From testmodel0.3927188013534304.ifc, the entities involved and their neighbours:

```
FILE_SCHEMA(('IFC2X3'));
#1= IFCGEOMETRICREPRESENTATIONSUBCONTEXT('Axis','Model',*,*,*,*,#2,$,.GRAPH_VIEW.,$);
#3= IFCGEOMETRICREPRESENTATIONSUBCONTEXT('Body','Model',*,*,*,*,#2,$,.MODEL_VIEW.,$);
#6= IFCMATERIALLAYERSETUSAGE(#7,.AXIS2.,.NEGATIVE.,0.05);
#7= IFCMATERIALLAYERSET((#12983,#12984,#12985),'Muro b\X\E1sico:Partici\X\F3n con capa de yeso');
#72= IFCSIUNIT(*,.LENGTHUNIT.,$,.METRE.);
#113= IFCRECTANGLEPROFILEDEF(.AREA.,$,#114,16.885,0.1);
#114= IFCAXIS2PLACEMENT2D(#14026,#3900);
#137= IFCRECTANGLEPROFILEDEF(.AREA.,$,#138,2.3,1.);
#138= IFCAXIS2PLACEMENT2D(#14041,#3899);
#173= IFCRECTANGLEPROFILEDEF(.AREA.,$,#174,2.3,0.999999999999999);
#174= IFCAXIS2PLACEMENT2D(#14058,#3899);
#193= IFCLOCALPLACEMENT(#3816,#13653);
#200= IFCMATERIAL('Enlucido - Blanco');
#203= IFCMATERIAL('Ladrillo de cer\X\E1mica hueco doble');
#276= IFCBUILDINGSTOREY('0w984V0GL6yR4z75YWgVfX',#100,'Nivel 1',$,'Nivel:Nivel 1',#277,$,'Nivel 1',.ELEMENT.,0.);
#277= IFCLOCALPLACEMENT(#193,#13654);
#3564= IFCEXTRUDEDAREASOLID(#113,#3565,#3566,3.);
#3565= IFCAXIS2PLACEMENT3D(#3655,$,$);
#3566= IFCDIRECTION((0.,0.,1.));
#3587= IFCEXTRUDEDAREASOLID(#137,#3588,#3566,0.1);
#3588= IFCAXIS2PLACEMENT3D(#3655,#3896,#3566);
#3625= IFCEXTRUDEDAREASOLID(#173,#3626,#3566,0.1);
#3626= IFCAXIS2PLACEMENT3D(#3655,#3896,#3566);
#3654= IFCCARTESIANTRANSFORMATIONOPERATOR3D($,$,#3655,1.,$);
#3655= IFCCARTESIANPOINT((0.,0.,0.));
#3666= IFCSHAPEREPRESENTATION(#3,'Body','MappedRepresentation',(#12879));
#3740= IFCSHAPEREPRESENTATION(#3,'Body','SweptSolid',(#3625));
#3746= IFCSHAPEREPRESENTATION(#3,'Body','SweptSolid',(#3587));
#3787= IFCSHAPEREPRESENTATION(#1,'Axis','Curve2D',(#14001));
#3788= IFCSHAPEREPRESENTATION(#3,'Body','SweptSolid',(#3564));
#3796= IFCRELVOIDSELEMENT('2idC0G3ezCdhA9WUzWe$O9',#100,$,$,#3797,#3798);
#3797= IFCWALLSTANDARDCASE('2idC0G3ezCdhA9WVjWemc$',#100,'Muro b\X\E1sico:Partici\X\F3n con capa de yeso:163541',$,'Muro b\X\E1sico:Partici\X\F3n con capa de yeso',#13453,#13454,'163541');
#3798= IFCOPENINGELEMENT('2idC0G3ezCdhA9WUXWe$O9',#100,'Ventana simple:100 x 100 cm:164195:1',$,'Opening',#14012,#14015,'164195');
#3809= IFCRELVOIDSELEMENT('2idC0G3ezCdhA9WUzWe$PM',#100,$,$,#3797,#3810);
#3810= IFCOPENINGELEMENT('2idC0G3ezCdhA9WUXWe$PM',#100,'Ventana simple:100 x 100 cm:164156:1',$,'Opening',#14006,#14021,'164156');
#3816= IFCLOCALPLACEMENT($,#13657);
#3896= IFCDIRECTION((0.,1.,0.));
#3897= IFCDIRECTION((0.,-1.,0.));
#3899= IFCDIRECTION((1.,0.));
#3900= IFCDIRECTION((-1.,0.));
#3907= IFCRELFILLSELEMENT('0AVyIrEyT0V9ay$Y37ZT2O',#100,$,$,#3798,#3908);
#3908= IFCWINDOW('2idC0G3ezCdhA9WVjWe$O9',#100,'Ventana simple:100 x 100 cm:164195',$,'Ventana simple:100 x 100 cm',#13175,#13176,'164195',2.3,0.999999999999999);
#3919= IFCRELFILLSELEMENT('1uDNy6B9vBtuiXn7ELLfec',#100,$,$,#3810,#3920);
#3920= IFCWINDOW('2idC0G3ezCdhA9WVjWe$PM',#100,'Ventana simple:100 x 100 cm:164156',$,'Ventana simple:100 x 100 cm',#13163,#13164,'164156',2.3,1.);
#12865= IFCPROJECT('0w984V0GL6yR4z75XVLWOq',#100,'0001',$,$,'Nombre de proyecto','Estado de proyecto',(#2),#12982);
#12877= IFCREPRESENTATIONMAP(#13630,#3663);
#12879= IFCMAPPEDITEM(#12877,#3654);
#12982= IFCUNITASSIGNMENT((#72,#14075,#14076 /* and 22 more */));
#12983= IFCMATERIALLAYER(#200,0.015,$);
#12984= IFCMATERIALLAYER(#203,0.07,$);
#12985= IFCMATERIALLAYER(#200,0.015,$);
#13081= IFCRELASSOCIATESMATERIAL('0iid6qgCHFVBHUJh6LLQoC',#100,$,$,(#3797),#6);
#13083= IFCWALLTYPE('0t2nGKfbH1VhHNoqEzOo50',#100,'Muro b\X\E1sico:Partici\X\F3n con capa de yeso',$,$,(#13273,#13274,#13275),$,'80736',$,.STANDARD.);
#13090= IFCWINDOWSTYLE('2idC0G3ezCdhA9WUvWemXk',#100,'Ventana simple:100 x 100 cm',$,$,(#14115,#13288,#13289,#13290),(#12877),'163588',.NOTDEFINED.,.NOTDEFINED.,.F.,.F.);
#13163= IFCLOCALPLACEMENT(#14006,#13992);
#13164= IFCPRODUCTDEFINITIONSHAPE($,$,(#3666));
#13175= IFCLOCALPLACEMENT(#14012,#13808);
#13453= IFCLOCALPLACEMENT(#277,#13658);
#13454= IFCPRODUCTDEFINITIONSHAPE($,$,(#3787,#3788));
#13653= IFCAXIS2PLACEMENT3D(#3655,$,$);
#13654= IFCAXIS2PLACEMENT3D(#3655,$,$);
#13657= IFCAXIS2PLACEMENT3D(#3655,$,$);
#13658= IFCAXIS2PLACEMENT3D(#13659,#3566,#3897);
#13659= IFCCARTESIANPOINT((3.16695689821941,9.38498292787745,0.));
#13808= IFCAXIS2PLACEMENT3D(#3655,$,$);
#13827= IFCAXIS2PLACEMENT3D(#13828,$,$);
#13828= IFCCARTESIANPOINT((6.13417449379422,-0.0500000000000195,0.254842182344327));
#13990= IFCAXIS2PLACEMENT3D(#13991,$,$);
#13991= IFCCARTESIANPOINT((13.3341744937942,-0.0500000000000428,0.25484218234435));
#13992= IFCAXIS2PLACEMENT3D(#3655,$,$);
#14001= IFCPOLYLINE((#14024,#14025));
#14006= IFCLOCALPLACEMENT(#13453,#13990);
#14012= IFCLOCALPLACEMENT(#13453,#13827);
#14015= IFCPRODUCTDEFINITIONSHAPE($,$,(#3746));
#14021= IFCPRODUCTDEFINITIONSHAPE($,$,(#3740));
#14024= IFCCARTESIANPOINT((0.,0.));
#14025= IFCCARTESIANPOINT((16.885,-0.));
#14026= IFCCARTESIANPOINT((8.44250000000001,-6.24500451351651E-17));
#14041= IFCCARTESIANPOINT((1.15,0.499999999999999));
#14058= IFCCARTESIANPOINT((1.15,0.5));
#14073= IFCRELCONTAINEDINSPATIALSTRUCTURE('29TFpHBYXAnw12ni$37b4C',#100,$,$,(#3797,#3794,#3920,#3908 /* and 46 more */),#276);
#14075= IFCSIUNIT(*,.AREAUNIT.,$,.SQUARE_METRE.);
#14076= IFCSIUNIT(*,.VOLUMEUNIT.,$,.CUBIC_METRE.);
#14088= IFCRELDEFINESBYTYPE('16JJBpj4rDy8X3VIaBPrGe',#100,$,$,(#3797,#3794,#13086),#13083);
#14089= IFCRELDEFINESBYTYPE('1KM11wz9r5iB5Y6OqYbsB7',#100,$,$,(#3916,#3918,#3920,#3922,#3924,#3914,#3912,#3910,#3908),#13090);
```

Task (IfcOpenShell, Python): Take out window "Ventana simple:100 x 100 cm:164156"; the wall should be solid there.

```python
import ifcopenshell
import ifcopenshell.api.feature
import ifcopenshell.api.root
import ifcopenshell.geom
import ifcopenshell.util.shape

model = ifcopenshell.open("testmodel0.3927188013534304.ifc")
settings = ifcopenshell.geom.settings()


def volume(element):
    """Net volume in cubic metres, openings subtracted."""
    shape = ifcopenshell.geom.create_shape(settings, element)
    return ifcopenshell.util.shape.get_volume(shape.geometry)


window = model.by_guid("2idC0G3ezCdhA9WVjWe$PM")
opening = window.FillsVoids[0].RelatingOpeningElement
wall = opening.VoidsElements[0].RelatingBuildingElement
before = volume(wall)

ifcopenshell.api.root.remove_product(model, product=window)
ifcopenshell.api.feature.remove_feature(model, feature=opening)

after = volume(wall)

print(f"wall volume {before:.3f} -> {after:.3f} m3")

model.write("testmodel0.3927188013534304-out.ifc")
```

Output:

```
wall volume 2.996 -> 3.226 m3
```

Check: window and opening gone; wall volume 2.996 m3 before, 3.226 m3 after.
